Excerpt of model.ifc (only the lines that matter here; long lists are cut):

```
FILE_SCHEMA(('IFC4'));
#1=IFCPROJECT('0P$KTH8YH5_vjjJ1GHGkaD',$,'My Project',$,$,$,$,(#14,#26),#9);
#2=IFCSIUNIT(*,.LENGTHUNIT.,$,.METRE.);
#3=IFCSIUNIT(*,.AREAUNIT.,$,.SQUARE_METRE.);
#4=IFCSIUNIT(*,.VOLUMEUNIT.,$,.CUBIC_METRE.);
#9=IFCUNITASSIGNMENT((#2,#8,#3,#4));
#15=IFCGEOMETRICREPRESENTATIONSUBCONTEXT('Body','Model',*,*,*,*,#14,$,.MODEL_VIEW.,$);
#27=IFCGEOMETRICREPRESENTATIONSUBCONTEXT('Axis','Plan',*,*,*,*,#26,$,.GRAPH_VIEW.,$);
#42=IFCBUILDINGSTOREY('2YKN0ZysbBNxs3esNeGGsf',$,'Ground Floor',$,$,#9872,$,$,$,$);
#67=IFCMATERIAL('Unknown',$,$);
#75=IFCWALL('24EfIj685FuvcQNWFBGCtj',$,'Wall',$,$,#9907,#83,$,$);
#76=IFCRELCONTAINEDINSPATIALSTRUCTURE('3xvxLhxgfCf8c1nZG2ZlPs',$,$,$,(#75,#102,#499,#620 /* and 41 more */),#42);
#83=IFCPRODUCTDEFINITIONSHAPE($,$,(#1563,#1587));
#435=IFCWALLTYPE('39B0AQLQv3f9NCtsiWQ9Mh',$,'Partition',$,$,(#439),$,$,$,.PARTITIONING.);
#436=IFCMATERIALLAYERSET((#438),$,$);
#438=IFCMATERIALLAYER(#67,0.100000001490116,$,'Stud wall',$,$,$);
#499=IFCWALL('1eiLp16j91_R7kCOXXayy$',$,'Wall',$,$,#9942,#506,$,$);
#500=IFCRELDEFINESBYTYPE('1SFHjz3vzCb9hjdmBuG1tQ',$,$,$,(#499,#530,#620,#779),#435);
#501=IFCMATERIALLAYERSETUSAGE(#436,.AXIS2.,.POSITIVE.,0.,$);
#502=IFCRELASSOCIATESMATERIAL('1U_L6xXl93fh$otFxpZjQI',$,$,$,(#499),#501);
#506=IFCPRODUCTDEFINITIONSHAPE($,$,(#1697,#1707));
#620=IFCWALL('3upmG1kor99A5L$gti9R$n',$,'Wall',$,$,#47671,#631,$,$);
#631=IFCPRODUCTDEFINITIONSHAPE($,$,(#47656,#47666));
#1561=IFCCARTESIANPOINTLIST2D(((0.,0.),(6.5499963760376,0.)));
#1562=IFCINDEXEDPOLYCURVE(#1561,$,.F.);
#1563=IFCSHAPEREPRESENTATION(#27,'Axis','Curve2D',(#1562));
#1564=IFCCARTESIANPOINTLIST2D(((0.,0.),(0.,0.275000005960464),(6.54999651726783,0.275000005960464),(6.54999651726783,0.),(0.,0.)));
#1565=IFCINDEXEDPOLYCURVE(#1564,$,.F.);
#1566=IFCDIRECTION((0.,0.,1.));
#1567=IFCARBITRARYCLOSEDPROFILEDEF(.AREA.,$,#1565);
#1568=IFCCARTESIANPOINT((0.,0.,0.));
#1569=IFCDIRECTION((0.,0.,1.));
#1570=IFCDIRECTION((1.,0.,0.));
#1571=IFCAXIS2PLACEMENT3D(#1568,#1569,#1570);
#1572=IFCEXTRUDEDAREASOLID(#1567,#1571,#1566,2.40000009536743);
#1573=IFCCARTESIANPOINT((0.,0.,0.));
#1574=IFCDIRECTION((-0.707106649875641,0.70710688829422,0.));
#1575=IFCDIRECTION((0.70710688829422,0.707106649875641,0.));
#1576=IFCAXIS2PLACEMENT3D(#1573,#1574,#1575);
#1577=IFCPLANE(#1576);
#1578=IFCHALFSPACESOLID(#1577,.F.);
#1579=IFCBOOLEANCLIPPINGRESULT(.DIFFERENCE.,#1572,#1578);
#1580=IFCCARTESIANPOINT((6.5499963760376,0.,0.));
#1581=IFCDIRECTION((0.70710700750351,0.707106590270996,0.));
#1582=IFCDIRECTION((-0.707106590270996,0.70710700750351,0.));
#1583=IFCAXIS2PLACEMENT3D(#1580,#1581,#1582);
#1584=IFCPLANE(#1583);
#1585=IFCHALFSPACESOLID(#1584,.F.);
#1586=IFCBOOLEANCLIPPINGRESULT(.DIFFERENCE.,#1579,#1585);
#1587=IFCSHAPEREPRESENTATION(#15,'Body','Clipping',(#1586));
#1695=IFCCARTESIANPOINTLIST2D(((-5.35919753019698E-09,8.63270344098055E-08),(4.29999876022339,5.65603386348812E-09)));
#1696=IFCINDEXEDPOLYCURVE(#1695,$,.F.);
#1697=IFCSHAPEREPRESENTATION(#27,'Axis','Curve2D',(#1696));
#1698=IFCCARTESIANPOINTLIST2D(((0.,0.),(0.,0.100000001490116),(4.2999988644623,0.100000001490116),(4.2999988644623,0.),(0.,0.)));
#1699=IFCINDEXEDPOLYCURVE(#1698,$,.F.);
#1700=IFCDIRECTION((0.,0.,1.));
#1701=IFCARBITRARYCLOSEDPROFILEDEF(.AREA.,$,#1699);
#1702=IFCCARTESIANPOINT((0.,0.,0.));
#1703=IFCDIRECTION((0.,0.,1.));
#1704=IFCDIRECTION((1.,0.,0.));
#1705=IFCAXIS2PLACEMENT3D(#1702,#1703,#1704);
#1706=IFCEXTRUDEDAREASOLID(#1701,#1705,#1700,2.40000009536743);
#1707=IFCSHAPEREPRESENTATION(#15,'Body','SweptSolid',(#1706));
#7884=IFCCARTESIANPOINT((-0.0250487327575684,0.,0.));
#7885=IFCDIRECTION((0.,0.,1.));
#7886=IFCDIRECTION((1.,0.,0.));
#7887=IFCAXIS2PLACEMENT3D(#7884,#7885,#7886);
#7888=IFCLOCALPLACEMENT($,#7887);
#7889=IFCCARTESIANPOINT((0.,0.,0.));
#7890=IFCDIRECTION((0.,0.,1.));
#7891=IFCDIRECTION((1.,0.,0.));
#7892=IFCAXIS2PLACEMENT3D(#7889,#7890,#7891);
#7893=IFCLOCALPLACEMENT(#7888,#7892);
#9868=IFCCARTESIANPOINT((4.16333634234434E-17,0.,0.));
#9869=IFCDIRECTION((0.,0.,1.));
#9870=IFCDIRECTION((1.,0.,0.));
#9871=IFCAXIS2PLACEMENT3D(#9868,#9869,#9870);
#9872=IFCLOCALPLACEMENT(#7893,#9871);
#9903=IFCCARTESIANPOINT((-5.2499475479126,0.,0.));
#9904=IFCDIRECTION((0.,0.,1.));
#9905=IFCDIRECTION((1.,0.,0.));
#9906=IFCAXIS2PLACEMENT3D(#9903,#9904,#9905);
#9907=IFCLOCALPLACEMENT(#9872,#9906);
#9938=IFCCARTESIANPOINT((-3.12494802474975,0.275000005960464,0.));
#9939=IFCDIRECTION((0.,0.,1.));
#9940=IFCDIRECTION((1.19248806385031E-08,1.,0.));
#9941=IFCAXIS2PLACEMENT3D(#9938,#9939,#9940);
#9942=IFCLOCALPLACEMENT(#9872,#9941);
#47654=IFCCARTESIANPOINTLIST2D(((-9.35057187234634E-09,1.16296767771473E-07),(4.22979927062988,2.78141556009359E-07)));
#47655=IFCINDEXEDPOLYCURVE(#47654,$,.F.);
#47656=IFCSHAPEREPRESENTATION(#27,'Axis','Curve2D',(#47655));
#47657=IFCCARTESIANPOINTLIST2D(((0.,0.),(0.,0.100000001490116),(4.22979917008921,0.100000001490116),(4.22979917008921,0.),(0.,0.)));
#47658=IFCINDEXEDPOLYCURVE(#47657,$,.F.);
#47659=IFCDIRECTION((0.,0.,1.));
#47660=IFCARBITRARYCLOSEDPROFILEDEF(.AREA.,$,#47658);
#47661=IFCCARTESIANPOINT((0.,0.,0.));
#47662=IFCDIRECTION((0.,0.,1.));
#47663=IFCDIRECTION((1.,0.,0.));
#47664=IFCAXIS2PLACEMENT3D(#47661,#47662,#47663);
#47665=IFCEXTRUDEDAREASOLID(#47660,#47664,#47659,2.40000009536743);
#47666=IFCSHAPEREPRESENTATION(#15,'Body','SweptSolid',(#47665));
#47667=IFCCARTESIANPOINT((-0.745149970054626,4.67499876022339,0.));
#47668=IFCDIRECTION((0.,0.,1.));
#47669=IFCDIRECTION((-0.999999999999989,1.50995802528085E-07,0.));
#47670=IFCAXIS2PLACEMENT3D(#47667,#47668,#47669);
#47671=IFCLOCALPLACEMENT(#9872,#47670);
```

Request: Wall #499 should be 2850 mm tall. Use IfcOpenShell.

```python
import ifcopenshell
import ifcopenshell.geom
import ifcopenshell.util.representation
import ifcopenshell.util.shape

model = ifcopenshell.open("model.ifc")
settings = ifcopenshell.geom.settings()


def volume(element):
    """Net volume in cubic metres, openings subtracted."""
    shape = ifcopenshell.geom.create_shape(settings, element)
    return ifcopenshell.util.shape.get_volume(shape.geometry)


wall = model.by_guid("1eiLp16j91_R7kCOXXayy$")
before = volume(wall)

body = ifcopenshell.util.representation.get_representation(wall, "Model", "Body")
solid = body.Items[0]
old_height = solid.Depth
solid.Depth = 2.85
after = volume(wall)

print(f"height {old_height:g} -> {solid.Depth:g}, volume {before:.3f} -> {after:.3f} m3")

model.write("model_edited.ifc")
```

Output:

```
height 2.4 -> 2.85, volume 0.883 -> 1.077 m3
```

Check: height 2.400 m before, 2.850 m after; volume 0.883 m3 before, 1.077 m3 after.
